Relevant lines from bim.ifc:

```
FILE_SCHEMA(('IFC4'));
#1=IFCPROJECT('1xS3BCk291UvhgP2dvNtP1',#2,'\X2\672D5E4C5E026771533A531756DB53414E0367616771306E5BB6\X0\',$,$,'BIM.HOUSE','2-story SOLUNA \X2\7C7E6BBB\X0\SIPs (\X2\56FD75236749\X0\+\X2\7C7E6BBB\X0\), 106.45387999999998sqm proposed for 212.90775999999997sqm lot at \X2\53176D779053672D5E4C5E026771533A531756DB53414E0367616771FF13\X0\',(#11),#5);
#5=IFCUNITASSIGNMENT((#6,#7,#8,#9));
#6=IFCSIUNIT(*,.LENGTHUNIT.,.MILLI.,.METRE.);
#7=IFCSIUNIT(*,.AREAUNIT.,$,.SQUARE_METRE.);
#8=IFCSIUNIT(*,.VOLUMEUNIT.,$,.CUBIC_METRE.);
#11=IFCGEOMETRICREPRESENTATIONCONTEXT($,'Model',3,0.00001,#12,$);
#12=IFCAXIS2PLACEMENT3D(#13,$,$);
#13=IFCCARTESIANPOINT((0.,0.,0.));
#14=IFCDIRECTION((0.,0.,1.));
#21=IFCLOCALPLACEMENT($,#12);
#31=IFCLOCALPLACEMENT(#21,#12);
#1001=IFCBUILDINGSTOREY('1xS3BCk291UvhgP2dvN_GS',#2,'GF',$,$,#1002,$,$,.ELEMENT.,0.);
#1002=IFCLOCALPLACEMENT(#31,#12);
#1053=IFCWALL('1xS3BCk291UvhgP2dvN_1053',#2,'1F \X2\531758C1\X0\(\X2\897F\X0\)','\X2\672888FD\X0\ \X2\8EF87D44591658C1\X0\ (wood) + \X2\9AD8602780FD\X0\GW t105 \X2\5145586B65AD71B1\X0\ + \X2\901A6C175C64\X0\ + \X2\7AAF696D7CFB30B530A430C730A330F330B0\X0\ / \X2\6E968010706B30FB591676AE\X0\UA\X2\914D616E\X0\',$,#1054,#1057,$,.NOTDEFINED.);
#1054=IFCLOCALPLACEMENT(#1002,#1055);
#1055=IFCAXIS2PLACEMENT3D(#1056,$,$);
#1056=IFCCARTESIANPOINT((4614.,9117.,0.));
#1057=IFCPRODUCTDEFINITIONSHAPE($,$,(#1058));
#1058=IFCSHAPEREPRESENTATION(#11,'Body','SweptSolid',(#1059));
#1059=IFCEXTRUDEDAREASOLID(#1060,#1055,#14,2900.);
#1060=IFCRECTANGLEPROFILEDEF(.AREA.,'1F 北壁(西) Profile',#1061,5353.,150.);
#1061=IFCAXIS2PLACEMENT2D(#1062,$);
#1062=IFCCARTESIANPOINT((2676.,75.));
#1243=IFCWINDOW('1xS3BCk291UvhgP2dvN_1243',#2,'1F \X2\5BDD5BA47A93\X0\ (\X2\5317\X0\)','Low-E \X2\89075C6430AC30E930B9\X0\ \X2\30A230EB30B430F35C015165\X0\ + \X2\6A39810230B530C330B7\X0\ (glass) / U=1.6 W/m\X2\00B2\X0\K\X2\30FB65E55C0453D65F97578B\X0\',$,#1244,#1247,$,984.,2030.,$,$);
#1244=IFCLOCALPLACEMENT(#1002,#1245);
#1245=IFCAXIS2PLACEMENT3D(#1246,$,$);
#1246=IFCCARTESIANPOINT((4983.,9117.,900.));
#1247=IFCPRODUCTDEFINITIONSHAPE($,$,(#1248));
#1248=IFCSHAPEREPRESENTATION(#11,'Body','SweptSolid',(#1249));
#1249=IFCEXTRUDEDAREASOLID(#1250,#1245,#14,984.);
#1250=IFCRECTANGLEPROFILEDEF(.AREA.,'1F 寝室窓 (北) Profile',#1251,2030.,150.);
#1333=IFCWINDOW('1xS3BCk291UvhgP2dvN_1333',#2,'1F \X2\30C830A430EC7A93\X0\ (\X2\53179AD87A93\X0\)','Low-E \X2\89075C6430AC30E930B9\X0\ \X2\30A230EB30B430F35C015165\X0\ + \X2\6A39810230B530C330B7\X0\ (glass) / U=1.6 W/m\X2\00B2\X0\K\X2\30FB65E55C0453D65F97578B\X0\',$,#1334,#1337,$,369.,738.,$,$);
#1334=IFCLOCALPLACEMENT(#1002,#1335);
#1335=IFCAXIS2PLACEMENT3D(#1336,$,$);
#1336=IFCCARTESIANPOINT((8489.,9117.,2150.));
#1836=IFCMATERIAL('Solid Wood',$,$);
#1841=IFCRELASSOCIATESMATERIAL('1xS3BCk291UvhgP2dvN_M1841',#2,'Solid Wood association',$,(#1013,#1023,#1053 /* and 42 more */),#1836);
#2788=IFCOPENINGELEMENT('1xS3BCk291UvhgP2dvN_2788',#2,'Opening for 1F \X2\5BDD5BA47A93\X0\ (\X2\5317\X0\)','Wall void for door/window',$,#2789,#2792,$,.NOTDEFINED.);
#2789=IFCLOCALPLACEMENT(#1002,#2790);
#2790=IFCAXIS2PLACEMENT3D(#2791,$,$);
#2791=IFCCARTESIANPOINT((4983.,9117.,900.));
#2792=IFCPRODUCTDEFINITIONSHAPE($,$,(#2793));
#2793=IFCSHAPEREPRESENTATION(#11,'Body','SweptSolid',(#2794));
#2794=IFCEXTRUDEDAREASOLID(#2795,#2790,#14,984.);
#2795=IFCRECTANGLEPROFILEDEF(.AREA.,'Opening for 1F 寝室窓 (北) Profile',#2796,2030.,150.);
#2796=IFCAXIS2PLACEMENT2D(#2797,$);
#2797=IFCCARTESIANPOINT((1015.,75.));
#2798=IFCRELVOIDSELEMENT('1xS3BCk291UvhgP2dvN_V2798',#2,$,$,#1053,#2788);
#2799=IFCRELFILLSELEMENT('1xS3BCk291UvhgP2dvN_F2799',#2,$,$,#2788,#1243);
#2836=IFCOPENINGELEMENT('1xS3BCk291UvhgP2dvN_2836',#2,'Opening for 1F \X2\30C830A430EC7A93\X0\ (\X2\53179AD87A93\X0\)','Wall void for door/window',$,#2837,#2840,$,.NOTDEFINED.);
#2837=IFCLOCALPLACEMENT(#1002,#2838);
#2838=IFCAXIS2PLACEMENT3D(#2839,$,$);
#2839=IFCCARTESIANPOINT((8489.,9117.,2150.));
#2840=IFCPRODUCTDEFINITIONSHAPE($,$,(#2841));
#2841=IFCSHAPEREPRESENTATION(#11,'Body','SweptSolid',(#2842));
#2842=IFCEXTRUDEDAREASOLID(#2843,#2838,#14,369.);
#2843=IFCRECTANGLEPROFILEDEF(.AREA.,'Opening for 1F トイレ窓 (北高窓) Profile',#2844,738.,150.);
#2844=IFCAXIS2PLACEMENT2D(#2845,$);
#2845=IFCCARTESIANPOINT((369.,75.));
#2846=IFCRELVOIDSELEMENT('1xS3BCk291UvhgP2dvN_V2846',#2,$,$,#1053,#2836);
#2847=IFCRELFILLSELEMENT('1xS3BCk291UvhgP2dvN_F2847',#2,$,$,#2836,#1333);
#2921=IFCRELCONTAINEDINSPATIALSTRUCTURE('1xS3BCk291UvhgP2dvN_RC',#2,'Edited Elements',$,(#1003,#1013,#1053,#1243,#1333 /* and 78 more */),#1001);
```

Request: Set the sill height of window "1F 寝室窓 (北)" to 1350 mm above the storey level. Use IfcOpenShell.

```python
import numpy as np
import ifcopenshell
import ifcopenshell.api.geometry
import ifcopenshell.geom
import ifcopenshell.util.element
import ifcopenshell.util.placement
import ifcopenshell.util.shape
import ifcopenshell.util.unit

model = ifcopenshell.open("bim.ifc")
unit_scale = ifcopenshell.util.unit.calculate_unit_scale(model)

window = model.by_guid("1xS3BCk291UvhgP2dvN_1243")
opening = window.FillsVoids[0].RelatingOpeningElement
storey = ifcopenshell.util.element.get_container(window, ifc_class="IfcBuildingStorey")
level = ifcopenshell.util.placement.get_local_placement(storey.ObjectPlacement)[2, 3]

# The opening's origin need not be at the sill, so measure its lowest point.
shape = ifcopenshell.geom.create_shape(ifcopenshell.geom.settings(), opening)
bottom = ifcopenshell.util.shape.get_shape_bottom_elevation(shape, shape.geometry) / unit_scale
dz = level + 1.35 / unit_scale - bottom

shift = np.array([0.0, 0.0, dz])
# The window is not placed relative to its opening, so move both.
for product in (opening, window):
    matrix = ifcopenshell.util.placement.get_local_placement(product.ObjectPlacement)
    matrix[:3, 3] += shift
    ifcopenshell.api.geometry.edit_object_placement(model, product=product, matrix=matrix, is_si=False)

print(f"moved by {dz * unit_scale:+.3f} m")

model.write("bim_edited.ifc")
```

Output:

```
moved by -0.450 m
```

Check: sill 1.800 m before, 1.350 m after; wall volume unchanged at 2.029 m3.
